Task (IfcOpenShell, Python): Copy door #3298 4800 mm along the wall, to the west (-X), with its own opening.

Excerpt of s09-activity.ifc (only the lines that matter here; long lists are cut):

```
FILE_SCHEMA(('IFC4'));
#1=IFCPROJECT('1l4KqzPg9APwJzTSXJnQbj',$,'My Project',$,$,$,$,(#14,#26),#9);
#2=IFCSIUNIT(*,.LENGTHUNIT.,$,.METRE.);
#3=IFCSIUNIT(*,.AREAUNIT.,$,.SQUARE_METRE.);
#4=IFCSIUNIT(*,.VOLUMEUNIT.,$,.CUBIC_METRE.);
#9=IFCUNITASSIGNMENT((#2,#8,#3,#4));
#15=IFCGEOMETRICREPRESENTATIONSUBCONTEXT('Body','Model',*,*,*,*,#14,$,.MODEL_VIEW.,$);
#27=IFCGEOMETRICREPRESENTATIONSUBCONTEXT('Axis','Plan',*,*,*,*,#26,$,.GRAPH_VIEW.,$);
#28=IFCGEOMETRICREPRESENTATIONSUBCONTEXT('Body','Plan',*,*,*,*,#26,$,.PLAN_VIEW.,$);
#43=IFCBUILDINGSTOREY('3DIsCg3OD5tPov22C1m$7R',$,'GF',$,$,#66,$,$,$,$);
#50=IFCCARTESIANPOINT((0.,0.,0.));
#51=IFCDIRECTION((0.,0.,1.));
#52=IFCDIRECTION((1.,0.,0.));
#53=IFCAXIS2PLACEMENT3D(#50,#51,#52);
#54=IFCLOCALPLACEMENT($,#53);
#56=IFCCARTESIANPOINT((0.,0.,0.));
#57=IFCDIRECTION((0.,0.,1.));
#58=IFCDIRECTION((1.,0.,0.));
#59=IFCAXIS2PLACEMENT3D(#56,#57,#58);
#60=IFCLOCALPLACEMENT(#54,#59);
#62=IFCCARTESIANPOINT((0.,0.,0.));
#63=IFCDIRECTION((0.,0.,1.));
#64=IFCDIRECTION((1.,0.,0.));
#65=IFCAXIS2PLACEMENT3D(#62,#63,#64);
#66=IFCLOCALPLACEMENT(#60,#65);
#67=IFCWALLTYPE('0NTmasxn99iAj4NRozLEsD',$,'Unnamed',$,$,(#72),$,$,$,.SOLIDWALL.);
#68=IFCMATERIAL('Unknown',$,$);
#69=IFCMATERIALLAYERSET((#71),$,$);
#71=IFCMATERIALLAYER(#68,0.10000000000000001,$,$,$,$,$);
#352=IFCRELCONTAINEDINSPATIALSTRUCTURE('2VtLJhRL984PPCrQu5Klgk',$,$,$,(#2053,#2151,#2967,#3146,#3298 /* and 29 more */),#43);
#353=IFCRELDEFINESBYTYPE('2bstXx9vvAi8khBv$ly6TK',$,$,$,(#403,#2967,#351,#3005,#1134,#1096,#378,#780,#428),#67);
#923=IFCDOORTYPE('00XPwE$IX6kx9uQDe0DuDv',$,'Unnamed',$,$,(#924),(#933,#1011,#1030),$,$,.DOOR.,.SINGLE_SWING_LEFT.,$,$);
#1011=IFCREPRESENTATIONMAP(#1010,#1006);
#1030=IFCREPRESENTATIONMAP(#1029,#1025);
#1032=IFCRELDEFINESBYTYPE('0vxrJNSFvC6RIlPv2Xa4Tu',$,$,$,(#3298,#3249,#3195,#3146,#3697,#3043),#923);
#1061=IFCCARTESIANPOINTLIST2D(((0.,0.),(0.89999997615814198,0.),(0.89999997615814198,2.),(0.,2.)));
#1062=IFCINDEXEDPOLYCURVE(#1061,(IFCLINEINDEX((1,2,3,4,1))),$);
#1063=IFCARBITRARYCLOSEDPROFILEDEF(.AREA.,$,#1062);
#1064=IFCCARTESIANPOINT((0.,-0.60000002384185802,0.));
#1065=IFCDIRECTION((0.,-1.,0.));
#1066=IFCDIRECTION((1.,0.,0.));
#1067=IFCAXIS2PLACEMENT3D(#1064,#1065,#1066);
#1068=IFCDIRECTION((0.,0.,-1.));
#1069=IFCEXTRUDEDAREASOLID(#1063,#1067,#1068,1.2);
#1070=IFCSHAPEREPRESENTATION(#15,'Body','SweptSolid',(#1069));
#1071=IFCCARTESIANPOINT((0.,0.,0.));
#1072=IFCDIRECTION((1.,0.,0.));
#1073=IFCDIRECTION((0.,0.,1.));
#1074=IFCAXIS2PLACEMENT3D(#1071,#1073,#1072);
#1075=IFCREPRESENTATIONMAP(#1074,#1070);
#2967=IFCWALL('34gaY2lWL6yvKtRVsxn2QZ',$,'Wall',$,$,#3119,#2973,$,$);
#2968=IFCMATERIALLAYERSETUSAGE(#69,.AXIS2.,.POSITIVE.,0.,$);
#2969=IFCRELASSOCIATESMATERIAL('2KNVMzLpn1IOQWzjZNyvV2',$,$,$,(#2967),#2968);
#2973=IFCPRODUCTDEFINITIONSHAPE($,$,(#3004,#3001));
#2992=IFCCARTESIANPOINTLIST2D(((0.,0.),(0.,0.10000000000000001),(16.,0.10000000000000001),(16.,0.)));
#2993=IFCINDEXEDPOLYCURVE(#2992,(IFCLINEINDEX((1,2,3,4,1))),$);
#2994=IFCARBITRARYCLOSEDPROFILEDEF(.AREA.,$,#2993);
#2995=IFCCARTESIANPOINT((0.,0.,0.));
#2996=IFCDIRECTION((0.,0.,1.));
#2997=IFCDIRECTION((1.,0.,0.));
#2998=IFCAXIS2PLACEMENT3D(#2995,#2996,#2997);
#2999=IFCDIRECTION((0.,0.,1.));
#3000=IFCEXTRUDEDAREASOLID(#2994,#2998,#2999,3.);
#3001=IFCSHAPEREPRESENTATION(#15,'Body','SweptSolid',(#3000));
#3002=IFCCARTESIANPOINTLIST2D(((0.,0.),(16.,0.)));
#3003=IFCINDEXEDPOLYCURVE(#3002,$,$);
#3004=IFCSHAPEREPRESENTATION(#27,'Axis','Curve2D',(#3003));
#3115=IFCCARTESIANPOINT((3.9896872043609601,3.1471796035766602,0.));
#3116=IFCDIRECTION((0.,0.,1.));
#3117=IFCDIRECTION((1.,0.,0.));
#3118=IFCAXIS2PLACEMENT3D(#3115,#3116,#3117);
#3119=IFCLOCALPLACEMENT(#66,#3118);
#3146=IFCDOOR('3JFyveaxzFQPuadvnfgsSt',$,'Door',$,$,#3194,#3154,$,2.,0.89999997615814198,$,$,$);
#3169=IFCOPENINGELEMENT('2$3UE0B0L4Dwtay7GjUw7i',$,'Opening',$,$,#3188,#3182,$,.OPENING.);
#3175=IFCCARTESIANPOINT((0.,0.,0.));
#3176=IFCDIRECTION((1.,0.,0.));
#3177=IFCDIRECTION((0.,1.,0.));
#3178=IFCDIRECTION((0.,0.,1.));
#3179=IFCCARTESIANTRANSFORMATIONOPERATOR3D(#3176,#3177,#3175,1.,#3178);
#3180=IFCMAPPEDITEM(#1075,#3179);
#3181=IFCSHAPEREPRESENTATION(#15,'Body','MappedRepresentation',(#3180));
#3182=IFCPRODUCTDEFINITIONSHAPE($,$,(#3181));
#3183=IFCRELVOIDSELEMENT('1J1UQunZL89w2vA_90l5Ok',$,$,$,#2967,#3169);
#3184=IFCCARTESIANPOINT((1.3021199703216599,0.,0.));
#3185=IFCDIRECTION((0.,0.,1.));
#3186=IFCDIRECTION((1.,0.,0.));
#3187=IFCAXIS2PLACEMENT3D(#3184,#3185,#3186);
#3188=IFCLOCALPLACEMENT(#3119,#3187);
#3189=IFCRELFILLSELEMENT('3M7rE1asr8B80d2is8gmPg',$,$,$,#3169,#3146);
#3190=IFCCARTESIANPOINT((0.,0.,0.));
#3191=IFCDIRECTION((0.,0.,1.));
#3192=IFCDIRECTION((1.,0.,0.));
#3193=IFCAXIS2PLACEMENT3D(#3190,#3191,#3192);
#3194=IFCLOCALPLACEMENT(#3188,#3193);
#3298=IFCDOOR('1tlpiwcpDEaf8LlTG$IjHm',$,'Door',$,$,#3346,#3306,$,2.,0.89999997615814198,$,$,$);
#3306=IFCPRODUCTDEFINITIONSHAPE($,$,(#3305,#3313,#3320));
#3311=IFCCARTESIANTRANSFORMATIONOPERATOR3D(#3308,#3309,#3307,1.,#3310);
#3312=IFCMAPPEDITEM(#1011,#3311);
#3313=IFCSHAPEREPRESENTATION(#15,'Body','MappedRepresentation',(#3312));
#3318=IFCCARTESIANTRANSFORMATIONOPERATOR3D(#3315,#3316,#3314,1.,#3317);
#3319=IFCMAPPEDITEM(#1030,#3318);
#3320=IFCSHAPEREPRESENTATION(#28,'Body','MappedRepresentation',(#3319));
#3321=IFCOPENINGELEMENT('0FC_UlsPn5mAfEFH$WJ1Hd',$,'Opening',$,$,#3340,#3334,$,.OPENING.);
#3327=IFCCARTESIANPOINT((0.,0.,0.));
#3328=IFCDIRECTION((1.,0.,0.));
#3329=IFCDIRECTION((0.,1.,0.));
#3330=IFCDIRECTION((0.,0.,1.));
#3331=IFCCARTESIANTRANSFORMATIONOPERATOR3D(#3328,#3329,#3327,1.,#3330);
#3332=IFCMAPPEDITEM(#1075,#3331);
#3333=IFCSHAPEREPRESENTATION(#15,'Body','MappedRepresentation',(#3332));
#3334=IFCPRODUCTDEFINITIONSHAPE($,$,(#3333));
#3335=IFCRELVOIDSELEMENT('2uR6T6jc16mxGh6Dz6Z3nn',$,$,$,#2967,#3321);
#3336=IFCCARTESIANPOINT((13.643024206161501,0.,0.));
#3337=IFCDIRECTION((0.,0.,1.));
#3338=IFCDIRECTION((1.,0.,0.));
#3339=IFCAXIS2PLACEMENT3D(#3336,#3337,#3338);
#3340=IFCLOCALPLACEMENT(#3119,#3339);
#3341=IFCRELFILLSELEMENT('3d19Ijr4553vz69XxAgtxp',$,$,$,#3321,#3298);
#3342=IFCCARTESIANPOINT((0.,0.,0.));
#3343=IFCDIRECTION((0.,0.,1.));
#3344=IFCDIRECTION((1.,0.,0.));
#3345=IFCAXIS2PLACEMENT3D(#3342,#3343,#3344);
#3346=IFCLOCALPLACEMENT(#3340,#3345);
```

```python
import ifcopenshell
import ifcopenshell.api.feature
import ifcopenshell.api.geometry
import ifcopenshell.api.root
import ifcopenshell.geom
import ifcopenshell.util.element
import ifcopenshell.util.placement
import ifcopenshell.util.shape
import ifcopenshell.util.unit

model = ifcopenshell.open("s09-activity.ifc")
unit_scale = ifcopenshell.util.unit.calculate_unit_scale(model)
settings = ifcopenshell.geom.settings()


def volume(element):
    """Net volume in cubic metres, openings subtracted."""
    shape = ifcopenshell.geom.create_shape(settings, element)
    return ifcopenshell.util.shape.get_volume(shape.geometry)


door = model.by_guid("1tlpiwcpDEaf8LlTG$IjHm")
opening = door.FillsVoids[0].RelatingOpeningElement
wall = opening.VoidsElements[0].RelatingBuildingElement
before = volume(wall)
shift = ifcopenshell.util.placement.get_local_placement(wall.ObjectPlacement)[:3, 0] * -4.8 / unit_scale

# copy_class copies the void relationship, type, container and properties, but no geometry.
new_opening = ifcopenshell.api.root.copy_class(model, product=opening)
new_opening.Representation = ifcopenshell.util.element.copy_deep(
    model, opening.Representation, exclude=["IfcGeometricRepresentationContext", "IfcRepresentationMap"]
)
new_door = ifcopenshell.api.root.copy_class(model, product=door)
new_door.Representation = ifcopenshell.util.element.copy_deep(
    model, door.Representation, exclude=["IfcGeometricRepresentationContext", "IfcRepresentationMap"]
)
ifcopenshell.api.feature.add_filling(model, opening=new_opening, element=new_door)

for old, new in ((opening, new_opening), (door, new_door)):
    matrix = ifcopenshell.util.placement.get_local_placement(old.ObjectPlacement)
    matrix[:3, 3] += shift
    ifcopenshell.api.geometry.edit_object_placement(model, product=new, matrix=matrix, is_si=False)

after = volume(wall)

print(f"wall volume {before:.3f} -> {after:.3f} m3")

model.write("s09-activity_edited.ifc")
```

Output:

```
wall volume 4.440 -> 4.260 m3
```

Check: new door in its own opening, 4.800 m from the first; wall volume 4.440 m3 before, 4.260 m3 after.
